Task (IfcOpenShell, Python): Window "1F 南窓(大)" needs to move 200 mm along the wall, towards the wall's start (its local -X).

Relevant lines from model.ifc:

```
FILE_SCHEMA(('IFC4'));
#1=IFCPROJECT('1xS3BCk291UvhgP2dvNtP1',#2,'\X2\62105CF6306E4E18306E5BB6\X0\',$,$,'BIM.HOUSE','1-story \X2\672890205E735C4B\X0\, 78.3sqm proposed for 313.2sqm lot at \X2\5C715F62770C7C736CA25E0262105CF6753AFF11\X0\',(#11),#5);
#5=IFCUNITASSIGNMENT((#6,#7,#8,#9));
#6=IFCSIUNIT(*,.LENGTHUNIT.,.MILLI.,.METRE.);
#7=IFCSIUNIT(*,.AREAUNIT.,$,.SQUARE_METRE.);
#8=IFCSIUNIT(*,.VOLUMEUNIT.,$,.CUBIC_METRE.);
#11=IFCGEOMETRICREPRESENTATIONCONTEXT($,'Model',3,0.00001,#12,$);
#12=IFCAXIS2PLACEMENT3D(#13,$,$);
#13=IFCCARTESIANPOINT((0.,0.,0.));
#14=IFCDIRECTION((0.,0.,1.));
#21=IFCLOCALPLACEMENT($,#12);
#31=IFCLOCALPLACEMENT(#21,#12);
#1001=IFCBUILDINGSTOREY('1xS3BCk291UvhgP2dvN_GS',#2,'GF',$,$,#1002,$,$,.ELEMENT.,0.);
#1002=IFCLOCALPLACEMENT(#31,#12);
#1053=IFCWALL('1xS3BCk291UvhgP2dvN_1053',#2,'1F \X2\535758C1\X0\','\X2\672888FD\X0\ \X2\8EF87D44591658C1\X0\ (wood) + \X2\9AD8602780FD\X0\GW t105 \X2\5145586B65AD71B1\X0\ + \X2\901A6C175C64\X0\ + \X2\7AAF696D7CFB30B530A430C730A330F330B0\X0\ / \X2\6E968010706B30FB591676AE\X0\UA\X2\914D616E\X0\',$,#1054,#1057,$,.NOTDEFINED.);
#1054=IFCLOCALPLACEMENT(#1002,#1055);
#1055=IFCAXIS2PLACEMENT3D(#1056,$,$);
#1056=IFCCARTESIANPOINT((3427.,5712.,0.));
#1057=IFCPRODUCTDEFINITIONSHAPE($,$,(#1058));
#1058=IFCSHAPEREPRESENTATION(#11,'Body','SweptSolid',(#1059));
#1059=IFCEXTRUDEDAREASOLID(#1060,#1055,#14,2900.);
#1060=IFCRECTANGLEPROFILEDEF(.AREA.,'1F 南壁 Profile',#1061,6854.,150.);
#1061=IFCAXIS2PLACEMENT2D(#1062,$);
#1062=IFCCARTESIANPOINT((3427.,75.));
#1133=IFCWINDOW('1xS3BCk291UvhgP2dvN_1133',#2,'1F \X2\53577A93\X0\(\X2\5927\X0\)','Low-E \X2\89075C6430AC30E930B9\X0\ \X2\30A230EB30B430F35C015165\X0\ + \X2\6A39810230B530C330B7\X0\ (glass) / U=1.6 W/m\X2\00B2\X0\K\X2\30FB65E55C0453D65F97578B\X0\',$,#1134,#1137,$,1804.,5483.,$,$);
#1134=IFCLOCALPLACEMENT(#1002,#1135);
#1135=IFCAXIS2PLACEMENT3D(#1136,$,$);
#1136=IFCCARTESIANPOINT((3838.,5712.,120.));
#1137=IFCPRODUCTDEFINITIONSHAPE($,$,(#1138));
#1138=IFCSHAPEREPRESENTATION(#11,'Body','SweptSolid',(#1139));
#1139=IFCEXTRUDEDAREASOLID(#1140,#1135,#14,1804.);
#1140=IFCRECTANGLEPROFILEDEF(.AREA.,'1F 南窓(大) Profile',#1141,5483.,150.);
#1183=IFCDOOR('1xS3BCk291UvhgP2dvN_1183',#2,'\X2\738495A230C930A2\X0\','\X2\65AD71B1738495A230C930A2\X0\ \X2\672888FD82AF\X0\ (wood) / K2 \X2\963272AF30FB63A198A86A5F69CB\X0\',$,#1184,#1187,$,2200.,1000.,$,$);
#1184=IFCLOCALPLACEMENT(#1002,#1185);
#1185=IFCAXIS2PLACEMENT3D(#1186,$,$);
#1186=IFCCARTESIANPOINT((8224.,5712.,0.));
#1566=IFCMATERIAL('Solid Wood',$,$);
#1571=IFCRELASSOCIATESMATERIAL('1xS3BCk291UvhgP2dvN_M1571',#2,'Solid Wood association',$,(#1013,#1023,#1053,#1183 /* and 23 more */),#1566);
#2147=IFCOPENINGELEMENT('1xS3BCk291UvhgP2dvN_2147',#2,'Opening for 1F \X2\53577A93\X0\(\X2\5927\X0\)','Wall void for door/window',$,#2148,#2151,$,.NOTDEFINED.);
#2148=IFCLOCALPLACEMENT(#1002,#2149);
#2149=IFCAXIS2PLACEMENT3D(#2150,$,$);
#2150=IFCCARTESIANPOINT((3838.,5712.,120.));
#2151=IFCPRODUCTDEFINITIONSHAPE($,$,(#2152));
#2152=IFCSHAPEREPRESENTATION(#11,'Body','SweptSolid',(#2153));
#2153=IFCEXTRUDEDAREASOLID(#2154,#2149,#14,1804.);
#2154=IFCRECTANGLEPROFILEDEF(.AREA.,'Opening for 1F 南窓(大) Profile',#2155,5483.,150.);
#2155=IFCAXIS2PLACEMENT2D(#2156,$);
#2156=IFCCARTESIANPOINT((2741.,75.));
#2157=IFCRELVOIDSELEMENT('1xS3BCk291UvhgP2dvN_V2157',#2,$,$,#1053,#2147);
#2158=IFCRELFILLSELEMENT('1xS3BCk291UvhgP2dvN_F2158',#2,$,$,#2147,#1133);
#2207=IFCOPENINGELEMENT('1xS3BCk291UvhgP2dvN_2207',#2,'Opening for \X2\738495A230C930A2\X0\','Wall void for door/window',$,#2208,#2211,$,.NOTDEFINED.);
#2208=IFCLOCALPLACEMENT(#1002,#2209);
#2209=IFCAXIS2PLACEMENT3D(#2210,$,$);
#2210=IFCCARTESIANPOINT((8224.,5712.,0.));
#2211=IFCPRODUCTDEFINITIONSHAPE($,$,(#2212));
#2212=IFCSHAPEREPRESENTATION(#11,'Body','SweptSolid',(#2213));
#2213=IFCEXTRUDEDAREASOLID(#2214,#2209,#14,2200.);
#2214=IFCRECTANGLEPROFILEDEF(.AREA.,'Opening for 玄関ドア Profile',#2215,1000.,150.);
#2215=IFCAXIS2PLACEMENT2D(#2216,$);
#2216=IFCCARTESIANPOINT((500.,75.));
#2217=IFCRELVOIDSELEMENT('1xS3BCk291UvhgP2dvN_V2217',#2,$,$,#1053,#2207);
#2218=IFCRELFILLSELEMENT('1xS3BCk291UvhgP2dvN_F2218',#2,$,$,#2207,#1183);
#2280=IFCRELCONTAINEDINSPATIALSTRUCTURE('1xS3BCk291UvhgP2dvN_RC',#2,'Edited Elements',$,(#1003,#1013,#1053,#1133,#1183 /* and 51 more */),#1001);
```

```python
import ifcopenshell
import ifcopenshell.api.geometry
import ifcopenshell.util.placement

model = ifcopenshell.open("model.ifc")

window = model.by_id(1133)
opening = window.FillsVoids[0].RelatingOpeningElement
wall = opening.VoidsElements[0].RelatingBuildingElement

wall_matrix = ifcopenshell.util.placement.get_local_placement(wall.ObjectPlacement)
shift = wall_matrix[:3, 0] * -200.0
before = ifcopenshell.util.placement.get_local_placement(window.ObjectPlacement)[:3, 3].copy()

# The window is not placed relative to its opening, so move both.
for product in (opening, window):
    matrix = ifcopenshell.util.placement.get_local_placement(product.ObjectPlacement)
    matrix[:3, 3] += shift
    ifcopenshell.api.geometry.edit_object_placement(model, product=product, matrix=matrix, is_si=False)

after = ifcopenshell.util.placement.get_local_placement(window.ObjectPlacement)[:3, 3]
print("window moved by", (after - before).round(3) + 0.0)

model.write("model_edited.ifc")
```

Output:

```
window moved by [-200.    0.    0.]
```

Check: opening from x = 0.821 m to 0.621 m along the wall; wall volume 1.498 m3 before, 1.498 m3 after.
